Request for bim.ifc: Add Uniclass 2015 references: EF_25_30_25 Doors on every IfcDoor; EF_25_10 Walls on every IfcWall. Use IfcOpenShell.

First a look at what the model holds.

```python
import ifcopenshell

model = ifcopenshell.open("bim.ifc")
print(model.schema)
print("classifications:", [c.Name for c in model.by_type("IfcClassification")])
for ifc_class in ("IfcDoor", "IfcRoof", "IfcStair", "IfcWall", "IfcWindow"):
    print(ifc_class, len(model.by_type(ifc_class)))
```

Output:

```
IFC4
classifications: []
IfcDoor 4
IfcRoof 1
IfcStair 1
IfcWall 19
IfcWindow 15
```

```python
import ifcopenshell
import ifcopenshell.api.classification

model = ifcopenshell.open("bim.ifc")

system = ifcopenshell.api.classification.add_classification(model, classification="Uniclass 2015")

codes = {
    "IfcDoor": ("EF_25_30_25", "Doors"),
    "IfcWall": ("EF_25_10", "Walls"),
}
for ifc_class, (code, name) in codes.items():
    products = model.by_type(ifc_class)
    ifcopenshell.api.classification.add_reference(
        model, products=products, classification=system, identification=code, name=name
    )
    print(code, len(products))

model.write("bim_v2.ifc")
```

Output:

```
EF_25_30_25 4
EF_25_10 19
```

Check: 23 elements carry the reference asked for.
